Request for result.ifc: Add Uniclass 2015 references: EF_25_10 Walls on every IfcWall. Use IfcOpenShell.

First a look at what the model holds.

```python
import ifcopenshell

model = ifcopenshell.open("result.ifc")
print(model.schema)
print("classifications:", [c.Name for c in model.by_type("IfcClassification")])
for ifc_class in ("IfcDoor", "IfcRoof", "IfcStair", "IfcWall", "IfcWindow"):
    print(ifc_class, len(model.by_type(ifc_class)))
```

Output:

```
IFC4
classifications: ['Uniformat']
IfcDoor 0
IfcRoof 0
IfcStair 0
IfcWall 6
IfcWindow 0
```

```python
import ifcopenshell
import ifcopenshell.api.classification

model = ifcopenshell.open("result.ifc")

system = ifcopenshell.api.classification.add_classification(model, classification="Uniclass 2015")

codes = {
    "IfcWall": ("EF_25_10", "Walls"),
}
for ifc_class, (code, name) in codes.items():
    products = model.by_type(ifc_class)
    ifcopenshell.api.classification.add_reference(
        model, products=products, classification=system, identification=code, name=name
    )
    print(code, len(products))

model.write("result_updated.ifc")
```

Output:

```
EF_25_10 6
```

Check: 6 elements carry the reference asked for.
